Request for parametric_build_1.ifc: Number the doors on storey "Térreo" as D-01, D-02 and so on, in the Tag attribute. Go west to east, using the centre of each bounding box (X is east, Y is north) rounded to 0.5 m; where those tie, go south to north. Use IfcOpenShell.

First a look at what the model holds.

```python
import ifcopenshell
import ifcopenshell.util.element
import ifcopenshell.util.placement

model = ifcopenshell.open("parametric_build_1.ifc")
print(model.schema)
storey = next(s for s in model.by_type("IfcBuildingStorey") if s.Name == "Térreo")
doors = [e for e in ifcopenshell.util.element.get_decomposition(storey) if e.is_a("IfcDoor")]
for e in sorted(doors, key=lambda e: e.id()):
    origin = ifcopenshell.util.placement.get_local_placement(e.ObjectPlacement)[:3, 3]
    print(e.id(), e.Tag, e.Name, origin.round(2) + 0.0, sep=" | ")
```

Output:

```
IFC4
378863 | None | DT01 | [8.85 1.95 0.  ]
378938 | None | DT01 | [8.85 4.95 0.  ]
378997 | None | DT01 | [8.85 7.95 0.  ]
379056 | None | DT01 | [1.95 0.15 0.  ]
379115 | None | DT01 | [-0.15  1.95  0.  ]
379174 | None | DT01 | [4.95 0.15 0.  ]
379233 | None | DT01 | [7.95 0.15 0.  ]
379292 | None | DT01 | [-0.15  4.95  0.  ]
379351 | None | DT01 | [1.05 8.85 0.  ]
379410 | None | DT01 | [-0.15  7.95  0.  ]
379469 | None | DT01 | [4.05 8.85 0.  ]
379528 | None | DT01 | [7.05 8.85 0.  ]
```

```python
import ifcopenshell
import ifcopenshell.geom
import ifcopenshell.util.element
import ifcopenshell.util.shape

model = ifcopenshell.open("parametric_build_1.ifc")
settings = ifcopenshell.geom.settings()
settings.set("use-world-coords", True)


def centre(element):
    shape = ifcopenshell.geom.create_shape(settings, element)
    return ifcopenshell.util.shape.get_bbox_centroid(shape.geometry)


storey = next(s for s in model.by_type("IfcBuildingStorey") if s.Name == "Térreo")
doors = [e for e in ifcopenshell.util.element.get_decomposition(storey) if e.is_a("IfcDoor")]

# Insertion points can sit at a corner or the storey origin, so sort by the geometry (in metres).
centres = {e: centre(e) for e in doors}
doors.sort(key=lambda e: (round(centres[e][0] / 0.5), centres[e][1]))

for i, e in enumerate(doors, start=1):
    number = f"D-{i:02d}"
    e.Tag = number
    print(e.id(), number)

model.write("parametric_build_1_edited.ifc")
```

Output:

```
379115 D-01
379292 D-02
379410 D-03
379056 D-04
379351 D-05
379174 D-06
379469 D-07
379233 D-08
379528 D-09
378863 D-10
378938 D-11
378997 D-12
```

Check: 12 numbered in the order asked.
